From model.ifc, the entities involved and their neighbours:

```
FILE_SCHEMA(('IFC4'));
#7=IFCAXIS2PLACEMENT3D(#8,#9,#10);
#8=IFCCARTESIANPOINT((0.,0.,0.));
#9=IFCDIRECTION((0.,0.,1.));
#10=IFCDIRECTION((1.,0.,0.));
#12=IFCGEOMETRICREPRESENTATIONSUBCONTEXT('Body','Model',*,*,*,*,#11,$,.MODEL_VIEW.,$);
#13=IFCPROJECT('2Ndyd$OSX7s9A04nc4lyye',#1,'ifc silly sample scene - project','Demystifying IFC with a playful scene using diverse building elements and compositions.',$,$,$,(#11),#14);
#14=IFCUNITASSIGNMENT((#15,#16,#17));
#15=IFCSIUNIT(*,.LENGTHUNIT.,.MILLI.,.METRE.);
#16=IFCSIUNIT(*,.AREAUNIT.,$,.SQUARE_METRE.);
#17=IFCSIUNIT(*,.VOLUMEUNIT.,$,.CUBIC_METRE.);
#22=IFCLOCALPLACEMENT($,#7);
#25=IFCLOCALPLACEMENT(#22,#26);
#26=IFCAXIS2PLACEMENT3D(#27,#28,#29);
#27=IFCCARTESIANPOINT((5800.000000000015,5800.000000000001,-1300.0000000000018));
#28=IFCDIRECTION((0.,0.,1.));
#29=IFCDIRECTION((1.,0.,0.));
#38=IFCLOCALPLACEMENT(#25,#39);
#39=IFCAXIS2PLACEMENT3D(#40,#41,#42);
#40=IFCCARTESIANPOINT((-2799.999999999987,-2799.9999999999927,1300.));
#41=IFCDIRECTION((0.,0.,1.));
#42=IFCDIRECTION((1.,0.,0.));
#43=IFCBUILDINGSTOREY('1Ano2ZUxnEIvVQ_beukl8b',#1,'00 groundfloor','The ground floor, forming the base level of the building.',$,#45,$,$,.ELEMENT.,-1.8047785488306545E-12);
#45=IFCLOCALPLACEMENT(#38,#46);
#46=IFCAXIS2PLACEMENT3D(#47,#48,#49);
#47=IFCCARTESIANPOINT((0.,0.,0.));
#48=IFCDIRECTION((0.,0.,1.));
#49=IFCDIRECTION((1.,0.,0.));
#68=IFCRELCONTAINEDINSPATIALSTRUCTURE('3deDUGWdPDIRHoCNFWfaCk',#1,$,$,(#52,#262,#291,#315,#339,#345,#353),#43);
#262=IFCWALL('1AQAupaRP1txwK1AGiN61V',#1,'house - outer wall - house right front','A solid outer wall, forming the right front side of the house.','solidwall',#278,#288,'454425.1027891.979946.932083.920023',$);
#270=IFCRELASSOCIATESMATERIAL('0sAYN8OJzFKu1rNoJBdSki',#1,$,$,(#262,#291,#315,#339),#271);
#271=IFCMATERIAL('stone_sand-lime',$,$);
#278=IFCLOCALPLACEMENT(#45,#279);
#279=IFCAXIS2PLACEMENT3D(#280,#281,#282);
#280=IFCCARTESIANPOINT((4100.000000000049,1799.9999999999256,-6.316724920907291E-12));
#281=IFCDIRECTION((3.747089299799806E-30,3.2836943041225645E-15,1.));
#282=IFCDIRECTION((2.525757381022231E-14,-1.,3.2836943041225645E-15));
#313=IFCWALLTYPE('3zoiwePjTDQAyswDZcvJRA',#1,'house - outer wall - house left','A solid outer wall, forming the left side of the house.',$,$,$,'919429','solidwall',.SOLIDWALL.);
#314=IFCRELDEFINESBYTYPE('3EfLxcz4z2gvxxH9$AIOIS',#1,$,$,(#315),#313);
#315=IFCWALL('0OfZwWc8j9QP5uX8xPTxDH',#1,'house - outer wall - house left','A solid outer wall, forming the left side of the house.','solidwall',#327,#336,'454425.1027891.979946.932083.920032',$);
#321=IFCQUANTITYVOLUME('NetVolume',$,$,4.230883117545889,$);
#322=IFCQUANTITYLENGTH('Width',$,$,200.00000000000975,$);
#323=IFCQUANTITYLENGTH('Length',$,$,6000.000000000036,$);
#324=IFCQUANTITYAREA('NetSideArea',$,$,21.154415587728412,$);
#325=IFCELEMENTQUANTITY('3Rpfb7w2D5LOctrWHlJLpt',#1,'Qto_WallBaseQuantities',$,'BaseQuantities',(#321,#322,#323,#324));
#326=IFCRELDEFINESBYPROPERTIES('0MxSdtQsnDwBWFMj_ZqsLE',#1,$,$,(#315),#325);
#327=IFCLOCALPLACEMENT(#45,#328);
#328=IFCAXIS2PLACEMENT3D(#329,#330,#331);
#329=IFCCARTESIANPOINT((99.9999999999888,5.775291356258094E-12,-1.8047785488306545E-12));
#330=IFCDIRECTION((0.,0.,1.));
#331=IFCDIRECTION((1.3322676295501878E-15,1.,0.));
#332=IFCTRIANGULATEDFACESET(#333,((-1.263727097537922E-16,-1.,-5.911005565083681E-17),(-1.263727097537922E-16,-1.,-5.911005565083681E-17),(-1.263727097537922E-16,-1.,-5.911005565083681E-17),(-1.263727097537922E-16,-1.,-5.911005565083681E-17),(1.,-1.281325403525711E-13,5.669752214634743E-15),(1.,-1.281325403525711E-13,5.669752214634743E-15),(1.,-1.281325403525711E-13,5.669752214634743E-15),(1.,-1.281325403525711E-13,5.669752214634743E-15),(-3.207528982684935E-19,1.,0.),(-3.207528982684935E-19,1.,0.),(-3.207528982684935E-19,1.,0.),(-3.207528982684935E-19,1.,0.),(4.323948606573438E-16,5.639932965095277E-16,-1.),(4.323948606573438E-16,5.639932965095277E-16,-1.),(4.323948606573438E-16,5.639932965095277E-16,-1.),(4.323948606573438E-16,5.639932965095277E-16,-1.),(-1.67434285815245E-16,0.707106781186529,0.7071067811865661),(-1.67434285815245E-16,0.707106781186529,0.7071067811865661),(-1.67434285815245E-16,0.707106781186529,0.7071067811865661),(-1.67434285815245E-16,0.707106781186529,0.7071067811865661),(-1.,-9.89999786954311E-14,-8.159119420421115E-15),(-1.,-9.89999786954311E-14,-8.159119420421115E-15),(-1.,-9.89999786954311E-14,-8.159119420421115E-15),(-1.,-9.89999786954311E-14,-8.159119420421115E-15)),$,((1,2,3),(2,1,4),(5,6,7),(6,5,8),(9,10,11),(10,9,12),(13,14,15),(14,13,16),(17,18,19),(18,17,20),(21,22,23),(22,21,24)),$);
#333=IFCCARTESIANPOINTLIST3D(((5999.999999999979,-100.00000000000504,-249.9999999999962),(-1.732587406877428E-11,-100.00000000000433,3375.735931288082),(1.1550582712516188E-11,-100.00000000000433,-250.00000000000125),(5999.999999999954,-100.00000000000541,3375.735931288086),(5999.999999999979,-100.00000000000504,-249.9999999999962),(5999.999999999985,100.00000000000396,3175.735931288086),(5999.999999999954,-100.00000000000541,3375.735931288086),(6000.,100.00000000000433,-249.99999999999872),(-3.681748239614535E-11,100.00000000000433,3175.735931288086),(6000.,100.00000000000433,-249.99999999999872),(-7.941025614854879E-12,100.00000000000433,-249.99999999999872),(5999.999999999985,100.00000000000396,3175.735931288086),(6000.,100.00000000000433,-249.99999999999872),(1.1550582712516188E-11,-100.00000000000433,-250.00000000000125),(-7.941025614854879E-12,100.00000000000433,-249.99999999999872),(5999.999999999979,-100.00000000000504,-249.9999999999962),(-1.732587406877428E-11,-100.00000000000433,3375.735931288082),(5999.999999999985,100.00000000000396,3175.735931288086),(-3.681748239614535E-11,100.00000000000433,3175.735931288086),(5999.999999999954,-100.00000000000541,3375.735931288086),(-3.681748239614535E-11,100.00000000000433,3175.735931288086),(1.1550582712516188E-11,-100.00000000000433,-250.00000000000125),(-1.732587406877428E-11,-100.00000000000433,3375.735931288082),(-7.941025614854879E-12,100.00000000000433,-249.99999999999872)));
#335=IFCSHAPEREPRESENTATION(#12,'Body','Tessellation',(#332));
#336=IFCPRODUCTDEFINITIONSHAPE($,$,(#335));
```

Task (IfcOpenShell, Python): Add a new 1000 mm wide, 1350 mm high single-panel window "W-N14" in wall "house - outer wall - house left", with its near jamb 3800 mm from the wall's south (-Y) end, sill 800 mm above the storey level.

```python
import numpy as np
import ifcopenshell
import ifcopenshell.api.feature
import ifcopenshell.api.geometry
import ifcopenshell.api.pset
import ifcopenshell.api.root
import ifcopenshell.api.spatial
import ifcopenshell.geom
import ifcopenshell.util.element
import ifcopenshell.util.placement
import ifcopenshell.util.representation
import ifcopenshell.util.shape
import ifcopenshell.util.unit

model = ifcopenshell.open("model.ifc")
unit_scale = ifcopenshell.util.unit.calculate_unit_scale(model)
area_scale = ifcopenshell.util.unit.calculate_unit_scale(model, "AREAUNIT")
volume_scale = ifcopenshell.util.unit.calculate_unit_scale(model, "VOLUMEUNIT")
settings = ifcopenshell.geom.settings()


def volume(element):
    """Net volume in cubic metres, openings subtracted."""
    shape = ifcopenshell.geom.create_shape(settings, element)
    return ifcopenshell.util.shape.get_volume(shape.geometry)


wall = model.by_guid("0OfZwWc8j9QP5uX8xPTxDH")
storey = ifcopenshell.util.element.get_container(wall, ifc_class="IfcBuildingStorey")
context = ifcopenshell.util.representation.get_context(model, "Model", "Body", "MODEL_VIEW")
before = volume(wall)

width, height, from_end, sill = 1, 1.35, 3.8, 0.8  # metres

# The wall runs along its own X axis, and the end named is its -X end.
wall_shape = ifcopenshell.geom.create_shape(settings, wall)
x, y, z = ifcopenshell.util.shape.get_vertices(wall_shape.geometry).T
start = x.min() + from_end
face, thickness = float(y.min()), float(y.max() - y.min())
wall_matrix = ifcopenshell.util.placement.get_local_placement(wall.ObjectPlacement)
level = ifcopenshell.util.placement.get_local_placement(storey.ObjectPlacement)[2, 3]


def in_wall(x, y):
    """Placement at x, y metres in the wall's axes, at sill height."""
    matrix = wall_matrix.copy()
    matrix[:, 3] = wall_matrix @ np.array([x / unit_scale, y / unit_scale, 0.0, 1.0])
    matrix[2, 3] = level + sill / unit_scale
    return matrix


# Opening: a box that overshoots both wall faces by 50 mm.
opening = ifcopenshell.api.root.create_entity(model, ifc_class="IfcOpeningElement", predefined_type="OPENING")
box = ifcopenshell.api.geometry.add_wall_representation(
    model, context=context, length=width, height=height, thickness=thickness + 0.1
)
ifcopenshell.api.geometry.assign_representation(model, product=opening, representation=box)
ifcopenshell.api.geometry.edit_object_placement(model, product=opening, matrix=in_wall(start, face - 0.05), is_si=False)
ifcopenshell.api.feature.add_feature(model, feature=opening, element=wall)

window = ifcopenshell.api.root.create_entity(model, ifc_class="IfcWindow", name="W-N14", predefined_type="WINDOW")
window.OverallWidth, window.OverallHeight = width / unit_scale, height / unit_scale
window.PartitioningType = "SINGLE_PANEL"
body = ifcopenshell.api.geometry.add_window_representation(
    model,
    context=context,
    overall_width=window.OverallWidth,
    overall_height=window.OverallHeight,
    partition_type="SINGLE_PANEL",
)
ifcopenshell.api.geometry.assign_representation(model, product=window, representation=body)
ifcopenshell.api.spatial.assign_container(model, products=[window], relating_structure=storey)
ifcopenshell.api.feature.add_filling(model, opening=opening, element=window)

# Centre the window in the wall's thickness.
ifcopenshell.api.geometry.edit_object_placement(model, product=window, matrix=in_wall(start, face), is_si=False)
window_shape = ifcopenshell.geom.create_shape(settings, window)
depth = ifcopenshell.util.shape.get_vertices(window_shape.geometry)[:, 1]
offset = face + thickness / 2 - (depth.min() + depth.max()) / 2
ifcopenshell.api.geometry.edit_object_placement(model, product=window, matrix=in_wall(start, offset), is_si=False)

after = volume(wall)

# Update the wall's stored quantities.
qto = model.by_id(ifcopenshell.util.element.get_pset(wall, "Qto_WallBaseQuantities", should_inherit=False)["id"])
ifcopenshell.api.pset.edit_qto(model, qto=qto, properties={
    "NetVolume": after / volume_scale,
    "NetSideArea": after / thickness / area_scale,
})

print(f"wall volume {before:.3f} -> {after:.3f} m3")

model.write("model_v2.ifc")
```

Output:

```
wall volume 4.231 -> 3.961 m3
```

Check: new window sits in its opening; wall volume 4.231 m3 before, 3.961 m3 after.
